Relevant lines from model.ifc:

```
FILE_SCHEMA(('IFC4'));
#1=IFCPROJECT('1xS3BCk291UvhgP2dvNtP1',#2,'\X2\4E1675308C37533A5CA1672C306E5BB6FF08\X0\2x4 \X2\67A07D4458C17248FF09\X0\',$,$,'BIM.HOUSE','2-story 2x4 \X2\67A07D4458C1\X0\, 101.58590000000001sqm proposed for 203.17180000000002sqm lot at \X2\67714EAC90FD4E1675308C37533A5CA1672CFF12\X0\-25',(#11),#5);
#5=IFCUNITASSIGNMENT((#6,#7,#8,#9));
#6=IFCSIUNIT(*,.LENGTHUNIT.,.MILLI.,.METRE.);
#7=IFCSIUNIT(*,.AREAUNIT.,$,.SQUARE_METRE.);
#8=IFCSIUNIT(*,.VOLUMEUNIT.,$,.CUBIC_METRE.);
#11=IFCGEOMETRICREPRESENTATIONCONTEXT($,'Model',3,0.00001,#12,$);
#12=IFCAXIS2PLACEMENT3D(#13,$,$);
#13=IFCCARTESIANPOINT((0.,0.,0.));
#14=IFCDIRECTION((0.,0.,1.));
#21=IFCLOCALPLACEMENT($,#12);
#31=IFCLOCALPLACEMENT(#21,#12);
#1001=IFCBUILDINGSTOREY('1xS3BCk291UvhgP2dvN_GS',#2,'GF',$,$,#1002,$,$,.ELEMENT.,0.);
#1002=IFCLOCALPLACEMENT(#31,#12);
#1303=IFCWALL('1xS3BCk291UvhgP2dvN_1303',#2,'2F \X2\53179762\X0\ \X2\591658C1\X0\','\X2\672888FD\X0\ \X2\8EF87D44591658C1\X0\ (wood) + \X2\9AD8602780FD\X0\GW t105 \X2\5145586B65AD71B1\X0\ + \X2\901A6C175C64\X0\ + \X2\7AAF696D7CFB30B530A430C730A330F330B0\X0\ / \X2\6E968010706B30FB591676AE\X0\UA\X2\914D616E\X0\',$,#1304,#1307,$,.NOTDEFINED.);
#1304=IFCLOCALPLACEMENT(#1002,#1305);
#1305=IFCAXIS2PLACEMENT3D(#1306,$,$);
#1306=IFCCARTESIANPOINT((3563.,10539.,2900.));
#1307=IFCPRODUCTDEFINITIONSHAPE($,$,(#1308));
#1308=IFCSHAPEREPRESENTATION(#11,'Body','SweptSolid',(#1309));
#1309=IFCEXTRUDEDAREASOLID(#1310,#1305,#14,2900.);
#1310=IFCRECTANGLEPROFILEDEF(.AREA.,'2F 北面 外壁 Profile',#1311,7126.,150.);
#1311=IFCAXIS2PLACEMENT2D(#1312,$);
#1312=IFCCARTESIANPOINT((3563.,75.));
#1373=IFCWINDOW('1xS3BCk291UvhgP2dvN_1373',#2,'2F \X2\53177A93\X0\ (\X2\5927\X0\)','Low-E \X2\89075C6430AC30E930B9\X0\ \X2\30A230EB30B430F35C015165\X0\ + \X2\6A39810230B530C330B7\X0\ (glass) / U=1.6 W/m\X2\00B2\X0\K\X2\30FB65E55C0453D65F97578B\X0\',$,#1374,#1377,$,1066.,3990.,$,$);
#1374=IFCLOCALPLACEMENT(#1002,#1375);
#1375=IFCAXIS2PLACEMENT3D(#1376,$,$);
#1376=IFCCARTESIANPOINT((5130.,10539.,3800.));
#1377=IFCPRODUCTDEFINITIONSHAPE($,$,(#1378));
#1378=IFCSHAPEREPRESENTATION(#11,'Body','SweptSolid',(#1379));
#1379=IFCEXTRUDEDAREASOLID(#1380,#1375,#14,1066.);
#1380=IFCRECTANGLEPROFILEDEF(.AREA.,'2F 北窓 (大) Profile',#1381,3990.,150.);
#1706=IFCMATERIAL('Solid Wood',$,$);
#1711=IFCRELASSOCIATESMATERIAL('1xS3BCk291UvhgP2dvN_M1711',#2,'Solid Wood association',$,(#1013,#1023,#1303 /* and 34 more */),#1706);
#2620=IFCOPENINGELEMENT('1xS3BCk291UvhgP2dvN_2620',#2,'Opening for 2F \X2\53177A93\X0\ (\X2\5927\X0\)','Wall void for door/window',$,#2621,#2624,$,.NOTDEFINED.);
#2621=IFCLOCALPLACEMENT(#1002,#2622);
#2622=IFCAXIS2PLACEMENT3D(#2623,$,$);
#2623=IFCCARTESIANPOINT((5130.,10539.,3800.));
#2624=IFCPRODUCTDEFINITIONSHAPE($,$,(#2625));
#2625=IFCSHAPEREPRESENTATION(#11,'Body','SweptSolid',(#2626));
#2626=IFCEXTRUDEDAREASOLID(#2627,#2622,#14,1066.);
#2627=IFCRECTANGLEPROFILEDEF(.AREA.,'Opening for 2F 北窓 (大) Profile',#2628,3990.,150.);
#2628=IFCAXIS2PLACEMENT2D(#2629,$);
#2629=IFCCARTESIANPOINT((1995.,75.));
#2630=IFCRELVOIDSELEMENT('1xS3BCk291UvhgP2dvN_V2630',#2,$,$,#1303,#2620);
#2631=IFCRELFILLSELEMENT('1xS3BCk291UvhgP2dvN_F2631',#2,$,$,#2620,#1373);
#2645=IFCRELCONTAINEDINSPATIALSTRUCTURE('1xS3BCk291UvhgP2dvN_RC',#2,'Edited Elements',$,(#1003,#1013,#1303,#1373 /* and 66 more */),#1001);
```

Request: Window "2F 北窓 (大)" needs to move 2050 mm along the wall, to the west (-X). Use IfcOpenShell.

```python
import ifcopenshell
import ifcopenshell.api.geometry
import ifcopenshell.util.placement
import ifcopenshell.util.unit

model = ifcopenshell.open("model.ifc")
unit_scale = ifcopenshell.util.unit.calculate_unit_scale(model)

window = model.by_guid("1xS3BCk291UvhgP2dvN_1373")
opening = window.FillsVoids[0].RelatingOpeningElement
wall = opening.VoidsElements[0].RelatingBuildingElement

wall_matrix = ifcopenshell.util.placement.get_local_placement(wall.ObjectPlacement)
shift = wall_matrix[:3, 0] * -2.05 / unit_scale
before = ifcopenshell.util.placement.get_local_placement(window.ObjectPlacement)[:3, 3].copy()

# The window is not placed relative to its opening, so move both.
for product in (opening, window):
    matrix = ifcopenshell.util.placement.get_local_placement(product.ObjectPlacement)
    matrix[:3, 3] += shift
    ifcopenshell.api.geometry.edit_object_placement(model, product=product, matrix=matrix, is_si=False)

after = ifcopenshell.util.placement.get_local_placement(window.ObjectPlacement)[:3, 3]
print("window moved by", (after - before).round(3) + 0.0)

model.write("model_rev.ifc")
```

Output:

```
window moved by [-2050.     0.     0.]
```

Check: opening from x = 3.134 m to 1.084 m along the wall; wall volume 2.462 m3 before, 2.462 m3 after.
